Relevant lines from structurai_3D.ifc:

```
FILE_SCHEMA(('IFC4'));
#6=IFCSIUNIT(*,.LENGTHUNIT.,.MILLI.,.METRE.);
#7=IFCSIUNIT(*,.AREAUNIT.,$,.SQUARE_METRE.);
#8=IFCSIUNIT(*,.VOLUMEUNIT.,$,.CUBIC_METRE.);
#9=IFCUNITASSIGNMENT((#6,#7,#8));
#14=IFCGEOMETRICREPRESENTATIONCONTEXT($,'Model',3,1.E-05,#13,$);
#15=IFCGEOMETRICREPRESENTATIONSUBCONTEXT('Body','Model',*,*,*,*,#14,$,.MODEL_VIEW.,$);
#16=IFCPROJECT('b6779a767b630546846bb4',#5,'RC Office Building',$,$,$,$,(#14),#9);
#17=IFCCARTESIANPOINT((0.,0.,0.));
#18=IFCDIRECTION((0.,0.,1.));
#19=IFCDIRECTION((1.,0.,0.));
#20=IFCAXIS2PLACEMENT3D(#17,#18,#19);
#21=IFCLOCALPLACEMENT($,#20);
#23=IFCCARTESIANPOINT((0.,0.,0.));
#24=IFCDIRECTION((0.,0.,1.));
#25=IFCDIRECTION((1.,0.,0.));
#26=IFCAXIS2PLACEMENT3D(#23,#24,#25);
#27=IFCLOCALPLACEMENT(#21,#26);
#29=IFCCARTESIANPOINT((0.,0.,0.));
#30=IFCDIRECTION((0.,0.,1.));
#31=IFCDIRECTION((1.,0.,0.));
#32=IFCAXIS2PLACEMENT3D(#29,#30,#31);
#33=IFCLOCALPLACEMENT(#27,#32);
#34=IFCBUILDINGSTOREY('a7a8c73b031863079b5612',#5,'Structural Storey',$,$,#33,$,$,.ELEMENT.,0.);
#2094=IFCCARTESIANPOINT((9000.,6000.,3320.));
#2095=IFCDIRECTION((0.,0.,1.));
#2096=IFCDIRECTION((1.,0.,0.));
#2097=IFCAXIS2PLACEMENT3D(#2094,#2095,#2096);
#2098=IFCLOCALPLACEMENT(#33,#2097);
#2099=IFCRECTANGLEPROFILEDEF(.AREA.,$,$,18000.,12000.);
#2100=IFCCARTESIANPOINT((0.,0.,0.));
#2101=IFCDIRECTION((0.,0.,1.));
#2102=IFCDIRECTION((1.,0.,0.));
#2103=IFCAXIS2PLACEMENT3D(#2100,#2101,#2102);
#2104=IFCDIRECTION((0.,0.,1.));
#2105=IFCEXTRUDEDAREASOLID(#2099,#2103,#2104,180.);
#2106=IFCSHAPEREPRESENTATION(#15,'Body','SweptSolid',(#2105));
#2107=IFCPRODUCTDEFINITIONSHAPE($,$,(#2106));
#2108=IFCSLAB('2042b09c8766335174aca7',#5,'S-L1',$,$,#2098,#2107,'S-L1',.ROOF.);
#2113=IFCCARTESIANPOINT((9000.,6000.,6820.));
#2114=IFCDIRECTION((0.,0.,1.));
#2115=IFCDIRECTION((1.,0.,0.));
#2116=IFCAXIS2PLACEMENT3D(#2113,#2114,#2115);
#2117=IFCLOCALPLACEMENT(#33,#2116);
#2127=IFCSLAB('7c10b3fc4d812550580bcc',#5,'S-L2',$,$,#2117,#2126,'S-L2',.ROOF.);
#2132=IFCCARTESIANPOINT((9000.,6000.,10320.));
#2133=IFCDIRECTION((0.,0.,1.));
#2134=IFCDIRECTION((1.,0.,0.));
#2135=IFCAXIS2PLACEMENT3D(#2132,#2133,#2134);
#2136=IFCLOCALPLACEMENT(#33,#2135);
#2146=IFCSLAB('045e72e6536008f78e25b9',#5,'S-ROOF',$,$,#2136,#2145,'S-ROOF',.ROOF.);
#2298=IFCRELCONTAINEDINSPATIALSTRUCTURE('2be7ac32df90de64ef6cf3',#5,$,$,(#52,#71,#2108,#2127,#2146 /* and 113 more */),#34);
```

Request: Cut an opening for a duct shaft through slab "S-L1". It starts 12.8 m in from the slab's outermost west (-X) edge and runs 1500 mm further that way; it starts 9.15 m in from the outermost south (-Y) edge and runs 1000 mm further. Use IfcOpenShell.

```python
import numpy as np
import ifcopenshell
import ifcopenshell.api.feature
import ifcopenshell.api.geometry
import ifcopenshell.api.root
import ifcopenshell.geom
import ifcopenshell.util.placement
import ifcopenshell.util.representation
import ifcopenshell.util.shape
import ifcopenshell.util.unit

model = ifcopenshell.open("structurai_3D.ifc")
unit_scale = ifcopenshell.util.unit.calculate_unit_scale(model)
settings = ifcopenshell.geom.settings()


def volume(element):
    """Net volume in cubic metres, openings subtracted."""
    shape = ifcopenshell.geom.create_shape(settings, element)
    return ifcopenshell.util.shape.get_volume(shape.geometry)


slab = model.by_id(2108)
before = volume(slab)

# Extent in the slab's own axes, in metres. The edges named are its -X and -Y sides.
slab_shape = ifcopenshell.geom.create_shape(settings, slab)
vertices = ifcopenshell.util.shape.get_vertices(slab_shape.geometry)
x_min, y_min, bottom = vertices.min(axis=0)
top = vertices[:, 2].max()

opening = ifcopenshell.api.root.create_entity(model, ifc_class="IfcOpeningElement", name="Duct shaft opening", predefined_type="OPENING")
context = ifcopenshell.util.representation.get_context(model, "Model", "Body", "MODEL_VIEW")
width, depth = 1.5, 1
outline = [(0.0, 0.0), (width, 0.0), (width, depth), (0.0, depth), (0.0, 0.0)]
# Overshoot both faces by 50 mm so the cut is clean.
shape = ifcopenshell.api.geometry.add_slab_representation(
    model, context=context, depth=top - bottom + 0.1, polyline=outline
)
ifcopenshell.api.geometry.assign_representation(model, product=opening, representation=shape)

matrix = ifcopenshell.util.placement.get_local_placement(slab.ObjectPlacement)
matrix[:, 3] = matrix @ np.append(np.array([x_min + 12.8, y_min + 9.15, bottom - 0.05]) / unit_scale, 1.0)
ifcopenshell.api.geometry.edit_object_placement(model, product=opening, matrix=matrix, is_si=False)
ifcopenshell.api.feature.add_feature(model, feature=opening, element=slab)

after = volume(slab)

print(f"slab volume {before:.3f} -> {after:.3f} m3")

model.write("structurai_3D_edited.ifc")
```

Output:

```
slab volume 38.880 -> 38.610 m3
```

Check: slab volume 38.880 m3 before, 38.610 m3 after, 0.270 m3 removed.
